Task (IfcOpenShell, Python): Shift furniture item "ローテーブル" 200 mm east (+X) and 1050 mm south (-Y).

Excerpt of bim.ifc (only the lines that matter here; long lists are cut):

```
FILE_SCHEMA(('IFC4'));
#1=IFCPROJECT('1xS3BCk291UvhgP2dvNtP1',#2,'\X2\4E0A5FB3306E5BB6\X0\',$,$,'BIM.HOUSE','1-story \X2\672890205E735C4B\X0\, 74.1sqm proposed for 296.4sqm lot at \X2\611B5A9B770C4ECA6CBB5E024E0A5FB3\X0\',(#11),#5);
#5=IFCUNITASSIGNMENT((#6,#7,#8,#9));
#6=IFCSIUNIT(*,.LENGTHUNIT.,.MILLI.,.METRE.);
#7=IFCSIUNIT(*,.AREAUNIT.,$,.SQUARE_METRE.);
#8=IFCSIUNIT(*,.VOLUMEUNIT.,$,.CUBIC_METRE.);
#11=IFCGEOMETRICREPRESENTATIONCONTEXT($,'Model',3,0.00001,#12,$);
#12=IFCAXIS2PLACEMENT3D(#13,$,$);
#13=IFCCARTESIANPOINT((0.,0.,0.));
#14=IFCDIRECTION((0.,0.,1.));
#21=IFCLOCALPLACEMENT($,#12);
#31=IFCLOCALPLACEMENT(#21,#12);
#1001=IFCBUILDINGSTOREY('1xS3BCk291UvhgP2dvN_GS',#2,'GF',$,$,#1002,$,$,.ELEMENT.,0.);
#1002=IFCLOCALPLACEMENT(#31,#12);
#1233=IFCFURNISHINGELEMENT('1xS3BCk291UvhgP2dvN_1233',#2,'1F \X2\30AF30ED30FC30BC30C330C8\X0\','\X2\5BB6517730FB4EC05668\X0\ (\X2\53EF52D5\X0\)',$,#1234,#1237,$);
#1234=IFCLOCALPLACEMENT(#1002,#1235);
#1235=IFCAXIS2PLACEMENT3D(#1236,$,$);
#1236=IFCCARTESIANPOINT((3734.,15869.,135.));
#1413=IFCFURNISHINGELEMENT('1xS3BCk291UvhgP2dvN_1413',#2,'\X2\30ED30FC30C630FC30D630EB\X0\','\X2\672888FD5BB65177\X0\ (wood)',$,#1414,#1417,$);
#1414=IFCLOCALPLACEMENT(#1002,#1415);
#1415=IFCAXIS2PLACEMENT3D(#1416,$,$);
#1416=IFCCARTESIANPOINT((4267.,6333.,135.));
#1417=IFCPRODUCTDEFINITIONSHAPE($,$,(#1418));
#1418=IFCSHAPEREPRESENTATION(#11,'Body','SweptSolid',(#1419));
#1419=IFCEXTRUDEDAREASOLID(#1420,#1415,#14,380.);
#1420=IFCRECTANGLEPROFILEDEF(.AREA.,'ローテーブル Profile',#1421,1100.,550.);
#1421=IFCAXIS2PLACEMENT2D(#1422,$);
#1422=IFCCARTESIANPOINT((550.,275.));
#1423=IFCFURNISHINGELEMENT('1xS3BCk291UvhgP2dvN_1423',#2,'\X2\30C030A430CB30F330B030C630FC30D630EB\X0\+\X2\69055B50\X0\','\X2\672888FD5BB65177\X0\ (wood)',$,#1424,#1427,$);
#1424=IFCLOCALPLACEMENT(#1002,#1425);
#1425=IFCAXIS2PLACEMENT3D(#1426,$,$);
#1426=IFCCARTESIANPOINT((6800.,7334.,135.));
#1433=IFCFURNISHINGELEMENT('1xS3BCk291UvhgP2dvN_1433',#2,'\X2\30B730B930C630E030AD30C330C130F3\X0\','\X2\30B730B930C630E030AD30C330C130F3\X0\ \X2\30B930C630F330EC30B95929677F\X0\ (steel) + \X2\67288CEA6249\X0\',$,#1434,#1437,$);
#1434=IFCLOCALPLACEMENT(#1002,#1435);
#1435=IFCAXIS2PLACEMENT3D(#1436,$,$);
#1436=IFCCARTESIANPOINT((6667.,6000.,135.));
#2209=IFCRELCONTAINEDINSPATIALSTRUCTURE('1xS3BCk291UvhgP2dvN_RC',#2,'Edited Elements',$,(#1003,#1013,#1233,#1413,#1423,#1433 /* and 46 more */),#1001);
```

```python
import ifcopenshell
import ifcopenshell.api.geometry
import ifcopenshell.util.placement
import ifcopenshell.util.unit

model = ifcopenshell.open("bim.ifc")
unit_scale = ifcopenshell.util.unit.calculate_unit_scale(model)

item = model.by_id(1413)
matrix = ifcopenshell.util.placement.get_local_placement(item.ObjectPlacement)
matrix[0, 3] += 0.2 / unit_scale
matrix[1, 3] -= 1.05 / unit_scale
ifcopenshell.api.geometry.edit_object_placement(model, product=item, matrix=matrix, is_si=False)

print(ifcopenshell.util.placement.get_local_placement(item.ObjectPlacement).round(3) + 0.0)

model.write("bim-out.ifc")
```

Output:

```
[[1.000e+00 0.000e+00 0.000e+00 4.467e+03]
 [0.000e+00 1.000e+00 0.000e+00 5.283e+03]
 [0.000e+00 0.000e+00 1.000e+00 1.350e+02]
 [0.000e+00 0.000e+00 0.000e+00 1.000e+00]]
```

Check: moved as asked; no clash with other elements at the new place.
